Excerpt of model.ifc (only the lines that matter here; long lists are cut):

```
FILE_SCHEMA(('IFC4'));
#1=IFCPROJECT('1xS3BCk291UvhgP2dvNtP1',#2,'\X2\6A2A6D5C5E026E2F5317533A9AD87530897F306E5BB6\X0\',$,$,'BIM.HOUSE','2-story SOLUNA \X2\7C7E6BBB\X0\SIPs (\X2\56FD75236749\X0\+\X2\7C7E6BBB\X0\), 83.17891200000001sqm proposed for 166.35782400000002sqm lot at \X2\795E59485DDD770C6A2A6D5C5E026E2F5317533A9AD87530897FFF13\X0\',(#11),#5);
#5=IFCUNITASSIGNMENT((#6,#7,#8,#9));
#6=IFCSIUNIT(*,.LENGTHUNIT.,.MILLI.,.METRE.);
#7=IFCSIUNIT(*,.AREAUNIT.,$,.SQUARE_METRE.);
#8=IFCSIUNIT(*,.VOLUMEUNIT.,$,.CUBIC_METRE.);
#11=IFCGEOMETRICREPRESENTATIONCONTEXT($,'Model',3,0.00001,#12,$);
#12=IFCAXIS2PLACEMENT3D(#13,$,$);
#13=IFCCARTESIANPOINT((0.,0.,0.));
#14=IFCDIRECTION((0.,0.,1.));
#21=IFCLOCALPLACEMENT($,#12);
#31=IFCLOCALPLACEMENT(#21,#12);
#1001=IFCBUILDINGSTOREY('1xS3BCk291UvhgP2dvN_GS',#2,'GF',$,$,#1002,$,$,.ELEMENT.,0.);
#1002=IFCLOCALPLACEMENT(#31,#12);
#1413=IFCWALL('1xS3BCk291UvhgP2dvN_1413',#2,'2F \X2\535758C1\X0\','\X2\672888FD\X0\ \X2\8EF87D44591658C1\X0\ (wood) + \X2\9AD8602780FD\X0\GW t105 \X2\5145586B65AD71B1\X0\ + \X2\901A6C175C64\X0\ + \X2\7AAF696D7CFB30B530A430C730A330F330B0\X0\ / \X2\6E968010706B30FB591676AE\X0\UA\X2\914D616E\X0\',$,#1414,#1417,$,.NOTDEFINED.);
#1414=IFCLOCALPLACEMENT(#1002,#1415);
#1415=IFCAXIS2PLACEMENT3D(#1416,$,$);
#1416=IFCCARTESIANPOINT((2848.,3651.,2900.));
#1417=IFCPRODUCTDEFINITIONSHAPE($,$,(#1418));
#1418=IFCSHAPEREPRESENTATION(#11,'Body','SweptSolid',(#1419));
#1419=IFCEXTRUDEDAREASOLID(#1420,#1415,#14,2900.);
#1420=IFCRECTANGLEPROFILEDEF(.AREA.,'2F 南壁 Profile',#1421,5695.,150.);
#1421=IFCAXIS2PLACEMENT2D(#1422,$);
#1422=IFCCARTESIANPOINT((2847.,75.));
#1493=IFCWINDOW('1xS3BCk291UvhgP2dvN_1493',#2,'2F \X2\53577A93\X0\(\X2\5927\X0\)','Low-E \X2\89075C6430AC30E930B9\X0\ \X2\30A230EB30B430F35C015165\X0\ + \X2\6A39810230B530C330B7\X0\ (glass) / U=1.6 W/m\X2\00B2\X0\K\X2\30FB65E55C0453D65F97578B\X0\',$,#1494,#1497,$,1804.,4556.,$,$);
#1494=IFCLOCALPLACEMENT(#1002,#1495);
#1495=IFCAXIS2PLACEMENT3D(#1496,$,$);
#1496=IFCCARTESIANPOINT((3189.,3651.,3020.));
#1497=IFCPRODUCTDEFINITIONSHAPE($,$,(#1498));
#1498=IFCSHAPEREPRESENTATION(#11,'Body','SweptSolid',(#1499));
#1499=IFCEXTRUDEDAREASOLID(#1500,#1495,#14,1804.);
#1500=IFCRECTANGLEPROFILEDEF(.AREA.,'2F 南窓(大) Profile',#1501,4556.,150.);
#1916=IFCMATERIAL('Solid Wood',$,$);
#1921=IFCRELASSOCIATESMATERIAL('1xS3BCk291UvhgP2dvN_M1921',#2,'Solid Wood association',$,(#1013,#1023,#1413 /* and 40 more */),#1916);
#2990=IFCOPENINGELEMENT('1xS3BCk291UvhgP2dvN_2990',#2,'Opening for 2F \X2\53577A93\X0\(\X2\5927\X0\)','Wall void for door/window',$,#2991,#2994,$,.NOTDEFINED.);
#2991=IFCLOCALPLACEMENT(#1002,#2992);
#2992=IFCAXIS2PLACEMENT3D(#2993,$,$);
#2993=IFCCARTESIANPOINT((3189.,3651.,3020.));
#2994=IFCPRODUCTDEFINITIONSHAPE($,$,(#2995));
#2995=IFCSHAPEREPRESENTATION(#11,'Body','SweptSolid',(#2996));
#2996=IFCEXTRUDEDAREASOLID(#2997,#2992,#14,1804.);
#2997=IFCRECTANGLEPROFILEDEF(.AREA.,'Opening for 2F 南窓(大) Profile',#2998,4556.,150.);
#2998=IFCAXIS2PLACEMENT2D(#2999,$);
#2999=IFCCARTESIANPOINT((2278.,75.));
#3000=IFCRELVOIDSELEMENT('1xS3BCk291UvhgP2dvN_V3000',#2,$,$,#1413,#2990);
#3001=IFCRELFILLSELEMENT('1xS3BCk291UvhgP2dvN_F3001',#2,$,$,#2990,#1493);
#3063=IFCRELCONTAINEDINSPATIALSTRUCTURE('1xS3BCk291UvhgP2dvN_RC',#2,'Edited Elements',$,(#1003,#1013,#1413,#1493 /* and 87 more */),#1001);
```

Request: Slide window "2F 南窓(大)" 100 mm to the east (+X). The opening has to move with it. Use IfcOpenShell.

```python
import ifcopenshell
import ifcopenshell.api.geometry
import ifcopenshell.util.placement
import ifcopenshell.util.unit

model = ifcopenshell.open("model.ifc")
unit_scale = ifcopenshell.util.unit.calculate_unit_scale(model)

window = model.by_guid("1xS3BCk291UvhgP2dvN_1493")
opening = window.FillsVoids[0].RelatingOpeningElement
wall = opening.VoidsElements[0].RelatingBuildingElement

wall_matrix = ifcopenshell.util.placement.get_local_placement(wall.ObjectPlacement)
shift = wall_matrix[:3, 0] * 0.1 / unit_scale
before = ifcopenshell.util.placement.get_local_placement(window.ObjectPlacement)[:3, 3].copy()

# The window is not placed relative to its opening, so move both.
for product in (opening, window):
    matrix = ifcopenshell.util.placement.get_local_placement(product.ObjectPlacement)
    matrix[:3, 3] += shift
    ifcopenshell.api.geometry.edit_object_placement(model, product=product, matrix=matrix, is_si=False)

after = ifcopenshell.util.placement.get_local_placement(window.ObjectPlacement)[:3, 3]
print("window moved by", (after - before).round(3) + 0.0)

model.write("model_v2.ifc")
```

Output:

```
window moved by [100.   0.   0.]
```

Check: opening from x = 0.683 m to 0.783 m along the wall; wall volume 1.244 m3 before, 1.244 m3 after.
